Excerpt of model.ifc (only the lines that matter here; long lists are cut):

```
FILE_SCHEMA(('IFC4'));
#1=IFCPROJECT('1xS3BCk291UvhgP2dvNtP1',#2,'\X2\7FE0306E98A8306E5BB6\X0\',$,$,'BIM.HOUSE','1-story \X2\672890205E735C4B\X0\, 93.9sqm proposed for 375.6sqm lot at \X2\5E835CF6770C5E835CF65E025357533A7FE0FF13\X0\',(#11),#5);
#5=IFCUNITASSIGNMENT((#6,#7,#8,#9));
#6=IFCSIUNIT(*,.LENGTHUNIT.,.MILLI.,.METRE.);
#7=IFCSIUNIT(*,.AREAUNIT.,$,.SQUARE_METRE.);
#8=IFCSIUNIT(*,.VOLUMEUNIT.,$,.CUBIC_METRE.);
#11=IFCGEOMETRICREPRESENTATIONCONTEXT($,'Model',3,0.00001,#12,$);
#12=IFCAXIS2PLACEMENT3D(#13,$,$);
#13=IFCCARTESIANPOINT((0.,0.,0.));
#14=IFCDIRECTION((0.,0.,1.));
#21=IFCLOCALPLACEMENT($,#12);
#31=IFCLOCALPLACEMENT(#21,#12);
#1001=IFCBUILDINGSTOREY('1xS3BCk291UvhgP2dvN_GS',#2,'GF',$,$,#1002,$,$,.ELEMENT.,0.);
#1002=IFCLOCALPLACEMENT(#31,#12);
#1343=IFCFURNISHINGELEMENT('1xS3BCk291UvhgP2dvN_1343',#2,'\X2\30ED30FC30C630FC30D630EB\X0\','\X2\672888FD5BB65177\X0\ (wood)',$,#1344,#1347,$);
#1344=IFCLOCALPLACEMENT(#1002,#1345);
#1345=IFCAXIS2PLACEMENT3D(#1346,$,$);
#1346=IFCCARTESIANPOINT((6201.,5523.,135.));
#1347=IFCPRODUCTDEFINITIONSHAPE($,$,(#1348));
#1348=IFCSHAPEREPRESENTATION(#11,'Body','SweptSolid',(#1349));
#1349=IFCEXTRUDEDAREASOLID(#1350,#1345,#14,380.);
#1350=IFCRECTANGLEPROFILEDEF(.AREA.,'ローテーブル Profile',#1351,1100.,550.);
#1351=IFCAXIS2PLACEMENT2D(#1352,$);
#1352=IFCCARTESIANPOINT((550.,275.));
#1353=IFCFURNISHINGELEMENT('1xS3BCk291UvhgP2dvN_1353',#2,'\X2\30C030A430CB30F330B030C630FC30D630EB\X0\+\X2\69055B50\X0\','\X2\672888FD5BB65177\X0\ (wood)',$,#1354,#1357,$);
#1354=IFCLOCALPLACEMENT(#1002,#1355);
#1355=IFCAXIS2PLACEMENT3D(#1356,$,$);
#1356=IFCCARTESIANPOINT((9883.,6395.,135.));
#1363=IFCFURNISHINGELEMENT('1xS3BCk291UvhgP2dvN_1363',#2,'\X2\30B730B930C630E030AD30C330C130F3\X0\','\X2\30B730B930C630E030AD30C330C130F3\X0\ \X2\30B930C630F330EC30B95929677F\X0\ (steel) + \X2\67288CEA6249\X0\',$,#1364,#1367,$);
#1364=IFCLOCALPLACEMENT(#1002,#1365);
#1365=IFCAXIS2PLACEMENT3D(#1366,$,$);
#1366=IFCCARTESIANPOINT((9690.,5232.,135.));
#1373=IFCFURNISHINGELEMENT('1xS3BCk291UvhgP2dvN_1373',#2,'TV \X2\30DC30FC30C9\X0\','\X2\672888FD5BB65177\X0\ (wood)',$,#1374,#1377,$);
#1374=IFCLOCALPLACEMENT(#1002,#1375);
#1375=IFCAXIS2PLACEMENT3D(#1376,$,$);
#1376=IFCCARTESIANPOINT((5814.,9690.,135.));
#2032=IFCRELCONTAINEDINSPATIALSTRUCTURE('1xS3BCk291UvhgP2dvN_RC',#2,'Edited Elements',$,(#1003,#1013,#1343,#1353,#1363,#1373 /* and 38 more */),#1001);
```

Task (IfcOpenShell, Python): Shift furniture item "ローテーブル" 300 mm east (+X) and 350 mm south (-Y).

```python
import ifcopenshell
import ifcopenshell.api.geometry
import ifcopenshell.util.placement

model = ifcopenshell.open("model.ifc")

item = model.by_guid("1xS3BCk291UvhgP2dvN_1343")
matrix = ifcopenshell.util.placement.get_local_placement(item.ObjectPlacement)
matrix[0, 3] += 300.0
matrix[1, 3] -= 350.0
ifcopenshell.api.geometry.edit_object_placement(model, product=item, matrix=matrix, is_si=False)

print(ifcopenshell.util.placement.get_local_placement(item.ObjectPlacement).round(3) + 0.0)

model.write("model_edited.ifc")
```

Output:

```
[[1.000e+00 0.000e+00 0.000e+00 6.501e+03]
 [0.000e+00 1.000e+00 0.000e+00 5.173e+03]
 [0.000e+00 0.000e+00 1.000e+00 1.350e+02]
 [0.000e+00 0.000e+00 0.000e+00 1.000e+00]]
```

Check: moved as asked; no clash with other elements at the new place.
